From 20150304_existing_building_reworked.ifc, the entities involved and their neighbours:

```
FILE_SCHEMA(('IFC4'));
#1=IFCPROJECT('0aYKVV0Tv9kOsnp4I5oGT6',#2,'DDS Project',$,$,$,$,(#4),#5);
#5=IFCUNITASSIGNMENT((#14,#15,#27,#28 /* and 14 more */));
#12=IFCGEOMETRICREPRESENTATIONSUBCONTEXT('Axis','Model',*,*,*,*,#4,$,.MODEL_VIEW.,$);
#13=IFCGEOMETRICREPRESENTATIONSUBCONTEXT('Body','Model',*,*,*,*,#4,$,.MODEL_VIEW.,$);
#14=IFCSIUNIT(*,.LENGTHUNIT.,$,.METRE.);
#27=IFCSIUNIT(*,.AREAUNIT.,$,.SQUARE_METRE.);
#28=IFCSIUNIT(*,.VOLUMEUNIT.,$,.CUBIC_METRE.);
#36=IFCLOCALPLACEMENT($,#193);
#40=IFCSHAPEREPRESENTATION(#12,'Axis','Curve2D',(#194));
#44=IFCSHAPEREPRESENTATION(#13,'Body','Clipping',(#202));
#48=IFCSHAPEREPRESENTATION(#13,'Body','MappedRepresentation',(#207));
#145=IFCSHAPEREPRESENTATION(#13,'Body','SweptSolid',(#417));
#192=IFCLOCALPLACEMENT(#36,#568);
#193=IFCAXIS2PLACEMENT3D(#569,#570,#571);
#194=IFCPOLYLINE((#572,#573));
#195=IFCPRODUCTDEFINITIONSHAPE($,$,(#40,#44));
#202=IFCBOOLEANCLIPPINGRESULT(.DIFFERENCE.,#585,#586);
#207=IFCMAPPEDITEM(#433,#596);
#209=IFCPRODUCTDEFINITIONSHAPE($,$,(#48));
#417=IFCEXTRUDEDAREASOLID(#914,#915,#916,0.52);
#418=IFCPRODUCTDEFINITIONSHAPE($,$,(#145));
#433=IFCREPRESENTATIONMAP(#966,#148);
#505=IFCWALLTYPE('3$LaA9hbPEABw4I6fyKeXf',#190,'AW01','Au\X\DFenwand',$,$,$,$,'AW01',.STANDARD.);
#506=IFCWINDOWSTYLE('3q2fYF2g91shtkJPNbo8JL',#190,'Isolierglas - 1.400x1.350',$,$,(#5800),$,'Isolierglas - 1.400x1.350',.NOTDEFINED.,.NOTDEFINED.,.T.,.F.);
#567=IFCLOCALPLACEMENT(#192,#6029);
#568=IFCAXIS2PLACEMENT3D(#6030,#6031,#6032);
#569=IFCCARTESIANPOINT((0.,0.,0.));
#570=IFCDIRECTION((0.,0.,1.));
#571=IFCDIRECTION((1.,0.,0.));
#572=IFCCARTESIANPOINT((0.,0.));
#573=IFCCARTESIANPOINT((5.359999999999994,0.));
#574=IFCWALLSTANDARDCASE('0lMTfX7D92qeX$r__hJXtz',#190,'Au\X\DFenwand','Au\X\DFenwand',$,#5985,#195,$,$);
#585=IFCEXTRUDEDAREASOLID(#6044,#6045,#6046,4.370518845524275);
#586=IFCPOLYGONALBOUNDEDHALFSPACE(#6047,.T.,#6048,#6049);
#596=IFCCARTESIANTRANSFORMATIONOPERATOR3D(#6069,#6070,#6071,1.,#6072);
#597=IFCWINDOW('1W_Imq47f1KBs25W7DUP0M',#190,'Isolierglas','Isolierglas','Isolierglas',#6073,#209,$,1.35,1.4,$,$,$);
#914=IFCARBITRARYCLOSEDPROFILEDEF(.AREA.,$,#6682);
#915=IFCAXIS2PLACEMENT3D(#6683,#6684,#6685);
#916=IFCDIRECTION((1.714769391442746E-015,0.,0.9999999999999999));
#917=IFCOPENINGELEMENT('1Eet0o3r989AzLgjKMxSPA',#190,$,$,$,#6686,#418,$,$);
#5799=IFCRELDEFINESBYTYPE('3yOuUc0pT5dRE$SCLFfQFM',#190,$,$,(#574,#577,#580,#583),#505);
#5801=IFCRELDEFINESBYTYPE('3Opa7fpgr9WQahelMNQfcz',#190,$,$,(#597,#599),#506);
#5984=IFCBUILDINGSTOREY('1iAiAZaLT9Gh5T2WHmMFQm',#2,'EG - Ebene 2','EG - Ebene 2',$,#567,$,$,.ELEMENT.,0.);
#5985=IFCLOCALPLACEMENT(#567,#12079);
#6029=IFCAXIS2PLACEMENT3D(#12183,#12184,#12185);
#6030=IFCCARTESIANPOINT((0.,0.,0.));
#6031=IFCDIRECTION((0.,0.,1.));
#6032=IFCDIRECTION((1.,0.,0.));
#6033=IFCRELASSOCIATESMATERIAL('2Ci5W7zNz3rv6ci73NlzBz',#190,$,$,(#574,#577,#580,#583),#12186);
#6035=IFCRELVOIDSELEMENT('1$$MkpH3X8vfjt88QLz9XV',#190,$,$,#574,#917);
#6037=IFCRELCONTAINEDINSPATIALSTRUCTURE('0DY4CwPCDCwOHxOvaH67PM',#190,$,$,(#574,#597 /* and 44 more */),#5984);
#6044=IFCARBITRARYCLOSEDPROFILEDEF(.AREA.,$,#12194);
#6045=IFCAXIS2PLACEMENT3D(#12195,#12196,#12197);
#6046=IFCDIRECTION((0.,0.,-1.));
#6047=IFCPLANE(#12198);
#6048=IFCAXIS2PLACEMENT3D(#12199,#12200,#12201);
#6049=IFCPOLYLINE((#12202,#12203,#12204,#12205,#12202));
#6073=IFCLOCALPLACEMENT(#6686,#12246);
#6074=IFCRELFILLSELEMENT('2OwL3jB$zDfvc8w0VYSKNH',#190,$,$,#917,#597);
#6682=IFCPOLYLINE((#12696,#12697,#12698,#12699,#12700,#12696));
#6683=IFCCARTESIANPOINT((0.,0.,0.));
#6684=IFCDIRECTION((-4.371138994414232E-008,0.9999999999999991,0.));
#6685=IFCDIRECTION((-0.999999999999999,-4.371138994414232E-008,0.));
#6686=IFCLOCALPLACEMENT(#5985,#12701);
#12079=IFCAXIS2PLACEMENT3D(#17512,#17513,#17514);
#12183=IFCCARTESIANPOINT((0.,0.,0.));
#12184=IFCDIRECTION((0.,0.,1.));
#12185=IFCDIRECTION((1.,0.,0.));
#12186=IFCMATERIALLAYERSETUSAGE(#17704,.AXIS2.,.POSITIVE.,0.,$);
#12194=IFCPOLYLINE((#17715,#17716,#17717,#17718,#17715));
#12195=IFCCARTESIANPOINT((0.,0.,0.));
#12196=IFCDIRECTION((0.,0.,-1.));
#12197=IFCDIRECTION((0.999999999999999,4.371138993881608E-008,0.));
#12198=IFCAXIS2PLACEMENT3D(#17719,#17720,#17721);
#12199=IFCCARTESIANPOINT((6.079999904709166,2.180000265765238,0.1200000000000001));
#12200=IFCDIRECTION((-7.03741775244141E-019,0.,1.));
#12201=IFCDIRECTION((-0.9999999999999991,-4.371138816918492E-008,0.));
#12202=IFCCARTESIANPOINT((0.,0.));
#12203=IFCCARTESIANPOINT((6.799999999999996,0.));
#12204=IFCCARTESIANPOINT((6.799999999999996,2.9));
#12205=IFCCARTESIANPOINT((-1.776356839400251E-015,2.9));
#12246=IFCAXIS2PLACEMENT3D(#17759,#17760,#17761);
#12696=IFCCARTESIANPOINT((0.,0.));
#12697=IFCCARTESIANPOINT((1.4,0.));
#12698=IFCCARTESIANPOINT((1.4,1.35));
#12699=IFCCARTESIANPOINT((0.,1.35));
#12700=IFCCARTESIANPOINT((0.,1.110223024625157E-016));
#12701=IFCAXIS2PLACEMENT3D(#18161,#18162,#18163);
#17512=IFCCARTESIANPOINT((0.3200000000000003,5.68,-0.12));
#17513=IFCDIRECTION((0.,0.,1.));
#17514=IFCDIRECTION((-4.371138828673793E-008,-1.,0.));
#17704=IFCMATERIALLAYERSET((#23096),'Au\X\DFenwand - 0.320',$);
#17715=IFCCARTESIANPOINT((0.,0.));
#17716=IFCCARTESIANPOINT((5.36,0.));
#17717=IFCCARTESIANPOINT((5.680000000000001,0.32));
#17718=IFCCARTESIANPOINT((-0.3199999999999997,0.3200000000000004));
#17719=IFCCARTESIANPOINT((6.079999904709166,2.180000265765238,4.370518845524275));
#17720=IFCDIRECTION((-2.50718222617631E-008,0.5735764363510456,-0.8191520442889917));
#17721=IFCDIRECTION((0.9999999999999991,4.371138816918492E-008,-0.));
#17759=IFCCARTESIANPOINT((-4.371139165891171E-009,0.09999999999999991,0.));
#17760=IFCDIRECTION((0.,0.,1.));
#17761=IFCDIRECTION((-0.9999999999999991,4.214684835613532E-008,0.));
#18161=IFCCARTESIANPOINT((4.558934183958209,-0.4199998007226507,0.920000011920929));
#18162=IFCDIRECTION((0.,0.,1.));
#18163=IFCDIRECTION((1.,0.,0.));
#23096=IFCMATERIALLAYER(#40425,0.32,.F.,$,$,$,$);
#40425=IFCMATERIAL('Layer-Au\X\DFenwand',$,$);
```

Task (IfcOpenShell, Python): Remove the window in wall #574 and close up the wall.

```python
import ifcopenshell
import ifcopenshell.api.feature
import ifcopenshell.api.root
import ifcopenshell.geom
import ifcopenshell.util.shape

model = ifcopenshell.open("20150304_existing_building_reworked.ifc")
settings = ifcopenshell.geom.settings()


def volume(element):
    """Net volume in cubic metres, openings subtracted."""
    shape = ifcopenshell.geom.create_shape(settings, element)
    return ifcopenshell.util.shape.get_volume(shape.geometry)


window = model.by_guid("1W_Imq47f1KBs25W7DUP0M")
opening = window.FillsVoids[0].RelatingOpeningElement
wall = opening.VoidsElements[0].RelatingBuildingElement
before = volume(wall)

ifcopenshell.api.root.remove_product(model, product=window)
ifcopenshell.api.feature.remove_feature(model, feature=opening)

after = volume(wall)

print(f"wall volume {before:.3f} -> {after:.3f} m3")

model.write("20150304_existing_building_reworked_rev.ifc")
```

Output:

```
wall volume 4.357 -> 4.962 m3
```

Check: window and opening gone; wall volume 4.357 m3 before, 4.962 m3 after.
